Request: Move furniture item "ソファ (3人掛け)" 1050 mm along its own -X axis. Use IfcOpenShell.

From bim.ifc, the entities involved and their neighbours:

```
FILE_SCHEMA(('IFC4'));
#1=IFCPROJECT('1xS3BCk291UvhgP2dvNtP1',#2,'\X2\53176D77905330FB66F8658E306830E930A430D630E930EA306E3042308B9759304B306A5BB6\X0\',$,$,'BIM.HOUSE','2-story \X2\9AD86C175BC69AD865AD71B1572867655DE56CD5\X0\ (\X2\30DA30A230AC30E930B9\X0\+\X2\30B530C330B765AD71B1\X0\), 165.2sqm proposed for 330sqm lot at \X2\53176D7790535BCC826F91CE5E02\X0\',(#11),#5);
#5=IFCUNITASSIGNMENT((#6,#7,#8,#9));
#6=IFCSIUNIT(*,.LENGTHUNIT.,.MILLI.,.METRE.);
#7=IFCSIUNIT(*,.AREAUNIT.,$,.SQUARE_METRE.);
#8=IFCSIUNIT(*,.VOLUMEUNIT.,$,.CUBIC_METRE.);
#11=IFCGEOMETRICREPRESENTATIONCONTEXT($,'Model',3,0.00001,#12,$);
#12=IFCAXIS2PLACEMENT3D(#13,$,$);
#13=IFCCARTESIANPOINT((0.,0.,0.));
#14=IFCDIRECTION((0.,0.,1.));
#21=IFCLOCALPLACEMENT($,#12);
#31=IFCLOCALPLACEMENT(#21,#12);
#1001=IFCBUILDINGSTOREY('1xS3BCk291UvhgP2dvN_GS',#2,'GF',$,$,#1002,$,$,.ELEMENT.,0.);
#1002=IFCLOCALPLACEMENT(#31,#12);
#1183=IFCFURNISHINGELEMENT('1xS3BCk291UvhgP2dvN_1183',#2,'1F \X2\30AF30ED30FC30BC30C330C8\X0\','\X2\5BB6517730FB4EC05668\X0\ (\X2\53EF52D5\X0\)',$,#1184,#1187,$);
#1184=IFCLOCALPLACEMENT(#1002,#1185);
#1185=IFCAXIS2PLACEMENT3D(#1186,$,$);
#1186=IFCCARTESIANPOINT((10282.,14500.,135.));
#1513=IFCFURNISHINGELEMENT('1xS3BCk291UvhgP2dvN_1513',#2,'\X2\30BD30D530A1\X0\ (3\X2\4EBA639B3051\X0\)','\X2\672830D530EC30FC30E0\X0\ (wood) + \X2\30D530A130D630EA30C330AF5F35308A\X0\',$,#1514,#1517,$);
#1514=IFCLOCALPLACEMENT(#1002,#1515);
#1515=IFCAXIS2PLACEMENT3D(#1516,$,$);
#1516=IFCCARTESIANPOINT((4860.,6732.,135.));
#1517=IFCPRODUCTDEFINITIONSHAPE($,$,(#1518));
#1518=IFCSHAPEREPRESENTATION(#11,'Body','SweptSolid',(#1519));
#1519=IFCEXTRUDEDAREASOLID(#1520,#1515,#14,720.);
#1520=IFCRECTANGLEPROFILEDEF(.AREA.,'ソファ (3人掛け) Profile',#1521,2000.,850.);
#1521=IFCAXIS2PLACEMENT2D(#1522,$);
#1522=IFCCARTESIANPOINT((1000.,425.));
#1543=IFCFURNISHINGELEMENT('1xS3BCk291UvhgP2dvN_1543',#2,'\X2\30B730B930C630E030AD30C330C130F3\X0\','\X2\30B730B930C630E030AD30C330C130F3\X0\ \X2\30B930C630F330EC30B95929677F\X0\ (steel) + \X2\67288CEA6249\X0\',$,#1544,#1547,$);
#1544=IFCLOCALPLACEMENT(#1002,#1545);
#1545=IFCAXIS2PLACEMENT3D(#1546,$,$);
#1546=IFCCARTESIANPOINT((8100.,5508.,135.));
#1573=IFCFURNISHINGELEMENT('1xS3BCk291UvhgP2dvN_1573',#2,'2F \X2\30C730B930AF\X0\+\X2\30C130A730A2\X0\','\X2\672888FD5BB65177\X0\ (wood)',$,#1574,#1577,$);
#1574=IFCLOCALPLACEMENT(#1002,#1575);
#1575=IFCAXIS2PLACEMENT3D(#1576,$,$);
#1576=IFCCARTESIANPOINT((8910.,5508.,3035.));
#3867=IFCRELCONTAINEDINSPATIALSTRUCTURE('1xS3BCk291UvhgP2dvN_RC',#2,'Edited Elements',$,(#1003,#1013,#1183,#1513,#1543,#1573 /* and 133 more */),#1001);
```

```python
import ifcopenshell
import ifcopenshell.api.geometry
import ifcopenshell.util.placement
import ifcopenshell.util.unit

model = ifcopenshell.open("bim.ifc")
unit_scale = ifcopenshell.util.unit.calculate_unit_scale(model)

item = model.by_guid("1xS3BCk291UvhgP2dvN_1513")
matrix = ifcopenshell.util.placement.get_local_placement(item.ObjectPlacement)
matrix[:3, 3] -= matrix[:3, 0] * 1.05 / unit_scale
ifcopenshell.api.geometry.edit_object_placement(model, product=item, matrix=matrix, is_si=False)

print(ifcopenshell.util.placement.get_local_placement(item.ObjectPlacement).round(3) + 0.0)

model.write("bim_edited.ifc")
```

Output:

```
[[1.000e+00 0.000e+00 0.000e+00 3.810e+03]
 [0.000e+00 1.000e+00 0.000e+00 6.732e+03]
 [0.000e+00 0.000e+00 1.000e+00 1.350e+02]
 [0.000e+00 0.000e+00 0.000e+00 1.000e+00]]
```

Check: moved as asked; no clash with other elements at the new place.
